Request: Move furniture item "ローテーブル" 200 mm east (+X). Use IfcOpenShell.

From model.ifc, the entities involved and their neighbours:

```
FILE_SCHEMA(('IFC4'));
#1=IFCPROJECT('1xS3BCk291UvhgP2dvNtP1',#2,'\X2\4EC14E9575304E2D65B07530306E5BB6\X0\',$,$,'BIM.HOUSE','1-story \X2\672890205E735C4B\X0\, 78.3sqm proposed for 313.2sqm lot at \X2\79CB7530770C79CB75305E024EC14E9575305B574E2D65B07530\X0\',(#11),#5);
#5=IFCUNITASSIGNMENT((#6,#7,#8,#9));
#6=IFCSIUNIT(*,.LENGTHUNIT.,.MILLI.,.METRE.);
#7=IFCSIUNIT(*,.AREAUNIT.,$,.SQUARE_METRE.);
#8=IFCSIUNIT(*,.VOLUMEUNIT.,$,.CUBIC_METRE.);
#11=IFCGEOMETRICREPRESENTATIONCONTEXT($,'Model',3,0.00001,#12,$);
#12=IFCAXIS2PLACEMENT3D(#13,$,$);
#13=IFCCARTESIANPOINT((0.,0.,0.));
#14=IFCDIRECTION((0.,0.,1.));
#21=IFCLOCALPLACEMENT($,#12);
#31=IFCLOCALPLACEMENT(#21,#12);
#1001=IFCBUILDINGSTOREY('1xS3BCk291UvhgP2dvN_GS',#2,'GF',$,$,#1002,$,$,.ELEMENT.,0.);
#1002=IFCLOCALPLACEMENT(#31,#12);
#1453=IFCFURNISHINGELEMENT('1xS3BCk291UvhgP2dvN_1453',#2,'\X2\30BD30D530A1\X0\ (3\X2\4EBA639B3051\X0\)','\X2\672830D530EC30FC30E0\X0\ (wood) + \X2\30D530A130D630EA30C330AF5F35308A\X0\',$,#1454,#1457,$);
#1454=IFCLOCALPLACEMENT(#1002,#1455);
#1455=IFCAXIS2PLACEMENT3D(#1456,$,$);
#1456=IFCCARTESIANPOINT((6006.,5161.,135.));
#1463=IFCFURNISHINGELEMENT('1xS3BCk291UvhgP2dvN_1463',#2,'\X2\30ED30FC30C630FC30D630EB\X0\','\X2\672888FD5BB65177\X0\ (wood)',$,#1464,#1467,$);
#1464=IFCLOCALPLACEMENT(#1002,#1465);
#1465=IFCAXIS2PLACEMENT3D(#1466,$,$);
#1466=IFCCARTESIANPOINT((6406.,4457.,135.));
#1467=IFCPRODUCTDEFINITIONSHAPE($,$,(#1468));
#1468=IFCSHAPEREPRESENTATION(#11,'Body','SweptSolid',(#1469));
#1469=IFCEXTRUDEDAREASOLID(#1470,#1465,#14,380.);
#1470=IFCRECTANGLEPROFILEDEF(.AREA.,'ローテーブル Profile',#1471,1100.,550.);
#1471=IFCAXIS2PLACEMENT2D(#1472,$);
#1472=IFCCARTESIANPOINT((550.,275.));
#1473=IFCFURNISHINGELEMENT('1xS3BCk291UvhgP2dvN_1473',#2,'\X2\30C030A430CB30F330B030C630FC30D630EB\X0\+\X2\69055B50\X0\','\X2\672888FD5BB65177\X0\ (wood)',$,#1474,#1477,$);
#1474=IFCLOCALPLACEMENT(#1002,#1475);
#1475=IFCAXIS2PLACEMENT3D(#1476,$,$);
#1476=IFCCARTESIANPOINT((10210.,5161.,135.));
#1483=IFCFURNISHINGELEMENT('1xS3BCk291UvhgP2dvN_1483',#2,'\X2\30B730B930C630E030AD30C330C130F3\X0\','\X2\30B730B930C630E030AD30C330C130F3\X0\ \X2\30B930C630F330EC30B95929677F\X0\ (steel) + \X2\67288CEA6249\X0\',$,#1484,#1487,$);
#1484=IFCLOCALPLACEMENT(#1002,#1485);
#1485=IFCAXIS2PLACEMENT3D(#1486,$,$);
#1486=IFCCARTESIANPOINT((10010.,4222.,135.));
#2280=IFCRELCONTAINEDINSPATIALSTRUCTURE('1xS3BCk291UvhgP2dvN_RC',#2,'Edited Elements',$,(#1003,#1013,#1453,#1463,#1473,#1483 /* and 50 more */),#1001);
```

```python
import ifcopenshell
import ifcopenshell.api.geometry
import ifcopenshell.util.placement
import ifcopenshell.util.unit

model = ifcopenshell.open("model.ifc")
unit_scale = ifcopenshell.util.unit.calculate_unit_scale(model)

item = model.by_guid("1xS3BCk291UvhgP2dvN_1463")
matrix = ifcopenshell.util.placement.get_local_placement(item.ObjectPlacement)
matrix[0, 3] += 0.2 / unit_scale
ifcopenshell.api.geometry.edit_object_placement(model, product=item, matrix=matrix, is_si=False)

print(ifcopenshell.util.placement.get_local_placement(item.ObjectPlacement).round(3) + 0.0)

model.write("model_rev.ifc")
```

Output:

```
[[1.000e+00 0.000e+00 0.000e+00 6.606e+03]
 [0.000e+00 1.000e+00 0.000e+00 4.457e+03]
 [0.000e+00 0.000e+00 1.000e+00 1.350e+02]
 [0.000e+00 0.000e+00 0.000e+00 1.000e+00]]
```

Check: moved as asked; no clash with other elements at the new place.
